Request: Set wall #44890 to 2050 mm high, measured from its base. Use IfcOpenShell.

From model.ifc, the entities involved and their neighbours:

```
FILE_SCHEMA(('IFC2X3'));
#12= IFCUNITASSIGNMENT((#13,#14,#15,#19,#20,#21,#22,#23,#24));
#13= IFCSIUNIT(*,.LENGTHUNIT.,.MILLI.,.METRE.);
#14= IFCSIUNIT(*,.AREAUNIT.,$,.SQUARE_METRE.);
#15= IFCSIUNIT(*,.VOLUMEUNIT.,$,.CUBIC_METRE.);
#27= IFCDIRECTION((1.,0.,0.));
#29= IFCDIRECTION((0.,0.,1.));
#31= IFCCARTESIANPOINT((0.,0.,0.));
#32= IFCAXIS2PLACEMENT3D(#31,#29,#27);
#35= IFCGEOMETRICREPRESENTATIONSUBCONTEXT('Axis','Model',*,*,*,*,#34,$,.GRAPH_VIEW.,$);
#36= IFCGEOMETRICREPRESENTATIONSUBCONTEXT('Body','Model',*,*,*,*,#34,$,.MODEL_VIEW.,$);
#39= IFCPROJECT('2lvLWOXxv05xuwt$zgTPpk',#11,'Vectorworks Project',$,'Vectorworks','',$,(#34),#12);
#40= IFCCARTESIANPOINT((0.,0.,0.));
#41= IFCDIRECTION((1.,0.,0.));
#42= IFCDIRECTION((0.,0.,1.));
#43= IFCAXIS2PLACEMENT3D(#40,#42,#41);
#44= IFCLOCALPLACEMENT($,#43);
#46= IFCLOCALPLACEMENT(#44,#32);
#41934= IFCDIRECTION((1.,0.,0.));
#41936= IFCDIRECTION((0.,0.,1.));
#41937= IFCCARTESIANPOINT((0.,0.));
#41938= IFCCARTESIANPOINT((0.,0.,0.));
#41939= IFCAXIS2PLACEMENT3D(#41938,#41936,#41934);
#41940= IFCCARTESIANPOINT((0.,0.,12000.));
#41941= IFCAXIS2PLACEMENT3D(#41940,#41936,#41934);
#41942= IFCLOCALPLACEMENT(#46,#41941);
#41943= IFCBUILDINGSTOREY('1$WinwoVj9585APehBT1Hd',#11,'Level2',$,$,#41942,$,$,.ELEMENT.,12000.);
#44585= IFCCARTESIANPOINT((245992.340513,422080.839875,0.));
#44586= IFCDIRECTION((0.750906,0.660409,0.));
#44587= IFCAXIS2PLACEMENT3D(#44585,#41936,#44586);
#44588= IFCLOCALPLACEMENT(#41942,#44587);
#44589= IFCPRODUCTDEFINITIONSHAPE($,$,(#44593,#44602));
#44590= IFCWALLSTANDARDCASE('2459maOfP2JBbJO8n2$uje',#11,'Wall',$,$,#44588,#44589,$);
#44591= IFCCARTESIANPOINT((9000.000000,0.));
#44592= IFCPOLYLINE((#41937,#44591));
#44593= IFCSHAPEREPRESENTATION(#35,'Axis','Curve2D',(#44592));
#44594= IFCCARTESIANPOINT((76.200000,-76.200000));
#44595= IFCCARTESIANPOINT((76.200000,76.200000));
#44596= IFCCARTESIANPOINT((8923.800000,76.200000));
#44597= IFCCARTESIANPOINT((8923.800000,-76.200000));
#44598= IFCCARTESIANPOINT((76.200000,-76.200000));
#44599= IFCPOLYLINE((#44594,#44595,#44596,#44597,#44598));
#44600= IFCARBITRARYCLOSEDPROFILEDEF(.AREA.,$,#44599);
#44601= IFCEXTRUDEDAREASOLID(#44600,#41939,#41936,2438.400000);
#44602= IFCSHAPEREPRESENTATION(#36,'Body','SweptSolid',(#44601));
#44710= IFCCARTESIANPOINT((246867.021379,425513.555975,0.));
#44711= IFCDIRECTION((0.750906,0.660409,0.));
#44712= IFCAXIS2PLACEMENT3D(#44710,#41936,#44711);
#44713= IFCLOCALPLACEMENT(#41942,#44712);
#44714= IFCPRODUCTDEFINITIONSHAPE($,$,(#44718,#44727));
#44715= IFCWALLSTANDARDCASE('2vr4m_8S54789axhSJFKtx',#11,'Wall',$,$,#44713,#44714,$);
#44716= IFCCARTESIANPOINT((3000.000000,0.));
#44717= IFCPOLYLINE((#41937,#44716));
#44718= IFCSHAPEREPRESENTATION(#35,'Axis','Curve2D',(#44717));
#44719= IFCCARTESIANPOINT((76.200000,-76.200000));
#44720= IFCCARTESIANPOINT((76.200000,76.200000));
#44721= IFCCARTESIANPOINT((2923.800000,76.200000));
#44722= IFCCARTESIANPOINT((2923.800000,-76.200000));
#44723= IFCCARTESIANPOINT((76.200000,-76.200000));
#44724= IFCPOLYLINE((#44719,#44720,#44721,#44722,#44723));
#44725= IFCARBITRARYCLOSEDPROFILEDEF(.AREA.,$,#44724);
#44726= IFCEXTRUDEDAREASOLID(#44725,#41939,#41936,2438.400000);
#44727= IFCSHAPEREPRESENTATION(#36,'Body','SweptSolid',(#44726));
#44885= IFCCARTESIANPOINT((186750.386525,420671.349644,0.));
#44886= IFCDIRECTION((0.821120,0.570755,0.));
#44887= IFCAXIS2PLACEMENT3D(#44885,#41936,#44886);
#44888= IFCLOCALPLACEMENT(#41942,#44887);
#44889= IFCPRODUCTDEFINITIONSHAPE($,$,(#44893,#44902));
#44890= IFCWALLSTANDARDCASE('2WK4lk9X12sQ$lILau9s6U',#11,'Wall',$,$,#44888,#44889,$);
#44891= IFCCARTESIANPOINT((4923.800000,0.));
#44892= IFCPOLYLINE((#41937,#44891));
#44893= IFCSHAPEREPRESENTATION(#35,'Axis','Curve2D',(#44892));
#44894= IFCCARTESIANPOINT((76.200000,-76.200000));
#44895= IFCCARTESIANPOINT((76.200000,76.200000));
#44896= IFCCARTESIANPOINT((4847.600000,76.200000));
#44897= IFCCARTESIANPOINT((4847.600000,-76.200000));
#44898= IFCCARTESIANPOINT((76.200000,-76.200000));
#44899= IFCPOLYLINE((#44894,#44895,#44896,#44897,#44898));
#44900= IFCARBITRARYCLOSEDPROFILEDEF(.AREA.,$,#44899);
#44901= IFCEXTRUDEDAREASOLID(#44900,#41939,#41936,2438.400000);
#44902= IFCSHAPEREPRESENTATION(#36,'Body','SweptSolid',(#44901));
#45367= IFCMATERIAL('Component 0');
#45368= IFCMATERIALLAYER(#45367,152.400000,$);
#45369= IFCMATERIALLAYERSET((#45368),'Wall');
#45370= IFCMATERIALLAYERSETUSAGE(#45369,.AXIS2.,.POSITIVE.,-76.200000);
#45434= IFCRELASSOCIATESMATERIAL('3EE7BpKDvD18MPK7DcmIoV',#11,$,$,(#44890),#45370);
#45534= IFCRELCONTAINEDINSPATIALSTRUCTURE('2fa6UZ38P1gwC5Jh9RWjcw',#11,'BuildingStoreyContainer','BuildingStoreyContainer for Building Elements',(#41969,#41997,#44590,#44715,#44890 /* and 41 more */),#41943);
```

```python
import ifcopenshell
import ifcopenshell.geom
import ifcopenshell.util.representation
import ifcopenshell.util.shape
import ifcopenshell.util.unit

model = ifcopenshell.open("model.ifc")
unit_scale = ifcopenshell.util.unit.calculate_unit_scale(model)
settings = ifcopenshell.geom.settings()


def volume(element):
    """Net volume in cubic metres, openings subtracted."""
    shape = ifcopenshell.geom.create_shape(settings, element)
    return ifcopenshell.util.shape.get_volume(shape.geometry)


wall = model.by_guid("2WK4lk9X12sQ$lILau9s6U")
before = volume(wall)

body = ifcopenshell.util.representation.get_representation(wall, "Model", "Body")
solid = body.Items[0]
old_height = solid.Depth
solid.Depth = 2.05 / unit_scale
after = volume(wall)

print(f"height {old_height:g} -> {solid.Depth:g}, volume {before:.3f} -> {after:.3f} m3")

model.write("model_edited.ifc")
```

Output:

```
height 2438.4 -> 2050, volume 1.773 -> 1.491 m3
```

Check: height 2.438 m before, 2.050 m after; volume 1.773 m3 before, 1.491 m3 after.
